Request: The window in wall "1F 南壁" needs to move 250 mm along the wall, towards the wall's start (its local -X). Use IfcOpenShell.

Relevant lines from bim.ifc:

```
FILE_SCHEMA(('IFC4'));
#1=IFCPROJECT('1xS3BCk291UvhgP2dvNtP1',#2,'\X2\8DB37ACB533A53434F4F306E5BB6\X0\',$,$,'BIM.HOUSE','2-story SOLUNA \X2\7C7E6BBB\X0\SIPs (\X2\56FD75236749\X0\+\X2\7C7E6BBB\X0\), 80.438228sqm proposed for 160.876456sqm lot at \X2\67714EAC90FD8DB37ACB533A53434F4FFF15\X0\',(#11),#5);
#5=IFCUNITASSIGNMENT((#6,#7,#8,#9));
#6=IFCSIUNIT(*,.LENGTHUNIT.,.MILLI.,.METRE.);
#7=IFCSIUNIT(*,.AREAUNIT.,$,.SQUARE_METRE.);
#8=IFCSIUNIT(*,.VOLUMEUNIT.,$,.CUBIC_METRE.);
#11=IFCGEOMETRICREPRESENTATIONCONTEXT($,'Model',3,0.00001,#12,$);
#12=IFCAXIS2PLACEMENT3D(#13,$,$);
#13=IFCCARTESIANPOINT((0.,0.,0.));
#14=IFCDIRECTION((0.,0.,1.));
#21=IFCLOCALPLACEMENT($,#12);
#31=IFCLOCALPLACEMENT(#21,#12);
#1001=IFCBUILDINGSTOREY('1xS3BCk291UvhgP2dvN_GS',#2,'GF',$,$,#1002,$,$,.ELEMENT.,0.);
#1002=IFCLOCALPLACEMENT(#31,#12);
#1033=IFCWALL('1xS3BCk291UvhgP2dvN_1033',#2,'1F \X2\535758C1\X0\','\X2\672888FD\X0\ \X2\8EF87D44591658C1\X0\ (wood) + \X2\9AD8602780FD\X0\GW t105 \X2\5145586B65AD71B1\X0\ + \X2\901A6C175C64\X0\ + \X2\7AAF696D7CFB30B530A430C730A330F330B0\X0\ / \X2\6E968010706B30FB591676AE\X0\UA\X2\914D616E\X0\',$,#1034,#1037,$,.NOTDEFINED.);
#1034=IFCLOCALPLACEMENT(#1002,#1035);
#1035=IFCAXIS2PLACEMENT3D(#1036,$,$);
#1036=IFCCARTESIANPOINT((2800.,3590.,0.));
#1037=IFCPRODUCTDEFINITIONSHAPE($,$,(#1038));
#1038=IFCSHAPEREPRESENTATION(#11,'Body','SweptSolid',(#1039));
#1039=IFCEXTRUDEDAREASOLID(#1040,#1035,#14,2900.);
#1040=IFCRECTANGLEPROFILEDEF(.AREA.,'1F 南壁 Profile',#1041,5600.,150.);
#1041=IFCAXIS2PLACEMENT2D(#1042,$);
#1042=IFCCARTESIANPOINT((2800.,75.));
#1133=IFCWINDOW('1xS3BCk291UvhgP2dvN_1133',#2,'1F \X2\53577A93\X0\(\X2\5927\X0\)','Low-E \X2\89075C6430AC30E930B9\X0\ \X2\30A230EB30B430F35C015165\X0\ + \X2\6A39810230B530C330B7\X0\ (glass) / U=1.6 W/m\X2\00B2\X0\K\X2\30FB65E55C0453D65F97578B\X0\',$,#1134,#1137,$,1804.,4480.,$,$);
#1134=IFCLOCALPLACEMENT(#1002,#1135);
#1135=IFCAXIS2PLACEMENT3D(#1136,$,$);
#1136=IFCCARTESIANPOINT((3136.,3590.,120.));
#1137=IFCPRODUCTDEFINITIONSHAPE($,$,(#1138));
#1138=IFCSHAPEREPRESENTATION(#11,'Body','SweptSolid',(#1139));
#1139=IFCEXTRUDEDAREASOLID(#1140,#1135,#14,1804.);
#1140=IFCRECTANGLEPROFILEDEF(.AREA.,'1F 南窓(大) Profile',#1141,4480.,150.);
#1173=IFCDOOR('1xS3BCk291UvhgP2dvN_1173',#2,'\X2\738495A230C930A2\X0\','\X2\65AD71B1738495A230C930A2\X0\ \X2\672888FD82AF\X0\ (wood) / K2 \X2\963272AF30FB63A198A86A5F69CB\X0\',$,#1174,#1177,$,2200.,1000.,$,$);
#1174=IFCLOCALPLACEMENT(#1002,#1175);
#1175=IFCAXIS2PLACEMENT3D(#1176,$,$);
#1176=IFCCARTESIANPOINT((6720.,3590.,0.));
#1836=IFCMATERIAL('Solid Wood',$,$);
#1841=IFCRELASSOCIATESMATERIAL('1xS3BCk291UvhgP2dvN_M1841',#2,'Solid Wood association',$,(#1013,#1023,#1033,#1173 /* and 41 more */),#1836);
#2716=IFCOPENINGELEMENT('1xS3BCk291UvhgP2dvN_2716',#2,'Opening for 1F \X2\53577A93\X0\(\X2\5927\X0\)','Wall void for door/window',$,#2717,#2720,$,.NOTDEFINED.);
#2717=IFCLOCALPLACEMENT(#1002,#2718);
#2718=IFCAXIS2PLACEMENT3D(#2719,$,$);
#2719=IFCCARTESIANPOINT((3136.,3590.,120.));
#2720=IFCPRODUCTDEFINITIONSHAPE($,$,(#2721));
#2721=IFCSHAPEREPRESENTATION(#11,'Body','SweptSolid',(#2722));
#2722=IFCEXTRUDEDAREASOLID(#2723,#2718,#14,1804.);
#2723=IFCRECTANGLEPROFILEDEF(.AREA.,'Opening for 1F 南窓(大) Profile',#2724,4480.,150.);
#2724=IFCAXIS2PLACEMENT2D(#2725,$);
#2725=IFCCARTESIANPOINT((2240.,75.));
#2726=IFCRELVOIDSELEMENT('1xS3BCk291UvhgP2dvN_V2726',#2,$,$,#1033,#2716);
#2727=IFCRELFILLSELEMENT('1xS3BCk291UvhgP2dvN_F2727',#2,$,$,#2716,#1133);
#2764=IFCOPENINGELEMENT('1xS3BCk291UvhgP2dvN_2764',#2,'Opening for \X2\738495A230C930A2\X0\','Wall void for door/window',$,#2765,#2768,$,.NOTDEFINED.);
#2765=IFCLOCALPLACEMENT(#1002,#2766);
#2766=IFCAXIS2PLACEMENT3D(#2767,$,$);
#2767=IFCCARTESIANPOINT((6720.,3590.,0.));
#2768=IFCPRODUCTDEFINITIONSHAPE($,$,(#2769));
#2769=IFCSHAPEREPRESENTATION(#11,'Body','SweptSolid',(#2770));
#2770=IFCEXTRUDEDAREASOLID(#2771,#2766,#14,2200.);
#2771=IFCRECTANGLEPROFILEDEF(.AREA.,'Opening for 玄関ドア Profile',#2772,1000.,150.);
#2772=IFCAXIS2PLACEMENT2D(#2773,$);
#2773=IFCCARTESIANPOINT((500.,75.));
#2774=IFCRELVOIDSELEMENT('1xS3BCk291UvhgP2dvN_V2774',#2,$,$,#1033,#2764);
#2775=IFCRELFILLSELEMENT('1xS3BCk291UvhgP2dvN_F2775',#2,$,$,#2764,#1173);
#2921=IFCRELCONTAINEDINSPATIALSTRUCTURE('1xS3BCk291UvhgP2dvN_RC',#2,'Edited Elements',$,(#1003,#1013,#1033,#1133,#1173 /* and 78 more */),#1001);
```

```python
import ifcopenshell
import ifcopenshell.api.geometry
import ifcopenshell.util.placement
import ifcopenshell.util.unit

model = ifcopenshell.open("bim.ifc")
unit_scale = ifcopenshell.util.unit.calculate_unit_scale(model)

window = model.by_guid("1xS3BCk291UvhgP2dvN_1133")
opening = window.FillsVoids[0].RelatingOpeningElement
wall = opening.VoidsElements[0].RelatingBuildingElement

wall_matrix = ifcopenshell.util.placement.get_local_placement(wall.ObjectPlacement)
shift = wall_matrix[:3, 0] * -0.25 / unit_scale
before = ifcopenshell.util.placement.get_local_placement(window.ObjectPlacement)[:3, 3].copy()

# The window is not placed relative to its opening, so move both.
for product in (opening, window):
    matrix = ifcopenshell.util.placement.get_local_placement(product.ObjectPlacement)
    matrix[:3, 3] += shift
    ifcopenshell.api.geometry.edit_object_placement(model, product=product, matrix=matrix, is_si=False)

after = ifcopenshell.util.placement.get_local_placement(window.ObjectPlacement)[:3, 3]
print("window moved by", (after - before).round(3) + 0.0)

model.write("bim_updated.ifc")
```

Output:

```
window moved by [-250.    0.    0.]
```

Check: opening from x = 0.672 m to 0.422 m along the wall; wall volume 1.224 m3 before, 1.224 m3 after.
